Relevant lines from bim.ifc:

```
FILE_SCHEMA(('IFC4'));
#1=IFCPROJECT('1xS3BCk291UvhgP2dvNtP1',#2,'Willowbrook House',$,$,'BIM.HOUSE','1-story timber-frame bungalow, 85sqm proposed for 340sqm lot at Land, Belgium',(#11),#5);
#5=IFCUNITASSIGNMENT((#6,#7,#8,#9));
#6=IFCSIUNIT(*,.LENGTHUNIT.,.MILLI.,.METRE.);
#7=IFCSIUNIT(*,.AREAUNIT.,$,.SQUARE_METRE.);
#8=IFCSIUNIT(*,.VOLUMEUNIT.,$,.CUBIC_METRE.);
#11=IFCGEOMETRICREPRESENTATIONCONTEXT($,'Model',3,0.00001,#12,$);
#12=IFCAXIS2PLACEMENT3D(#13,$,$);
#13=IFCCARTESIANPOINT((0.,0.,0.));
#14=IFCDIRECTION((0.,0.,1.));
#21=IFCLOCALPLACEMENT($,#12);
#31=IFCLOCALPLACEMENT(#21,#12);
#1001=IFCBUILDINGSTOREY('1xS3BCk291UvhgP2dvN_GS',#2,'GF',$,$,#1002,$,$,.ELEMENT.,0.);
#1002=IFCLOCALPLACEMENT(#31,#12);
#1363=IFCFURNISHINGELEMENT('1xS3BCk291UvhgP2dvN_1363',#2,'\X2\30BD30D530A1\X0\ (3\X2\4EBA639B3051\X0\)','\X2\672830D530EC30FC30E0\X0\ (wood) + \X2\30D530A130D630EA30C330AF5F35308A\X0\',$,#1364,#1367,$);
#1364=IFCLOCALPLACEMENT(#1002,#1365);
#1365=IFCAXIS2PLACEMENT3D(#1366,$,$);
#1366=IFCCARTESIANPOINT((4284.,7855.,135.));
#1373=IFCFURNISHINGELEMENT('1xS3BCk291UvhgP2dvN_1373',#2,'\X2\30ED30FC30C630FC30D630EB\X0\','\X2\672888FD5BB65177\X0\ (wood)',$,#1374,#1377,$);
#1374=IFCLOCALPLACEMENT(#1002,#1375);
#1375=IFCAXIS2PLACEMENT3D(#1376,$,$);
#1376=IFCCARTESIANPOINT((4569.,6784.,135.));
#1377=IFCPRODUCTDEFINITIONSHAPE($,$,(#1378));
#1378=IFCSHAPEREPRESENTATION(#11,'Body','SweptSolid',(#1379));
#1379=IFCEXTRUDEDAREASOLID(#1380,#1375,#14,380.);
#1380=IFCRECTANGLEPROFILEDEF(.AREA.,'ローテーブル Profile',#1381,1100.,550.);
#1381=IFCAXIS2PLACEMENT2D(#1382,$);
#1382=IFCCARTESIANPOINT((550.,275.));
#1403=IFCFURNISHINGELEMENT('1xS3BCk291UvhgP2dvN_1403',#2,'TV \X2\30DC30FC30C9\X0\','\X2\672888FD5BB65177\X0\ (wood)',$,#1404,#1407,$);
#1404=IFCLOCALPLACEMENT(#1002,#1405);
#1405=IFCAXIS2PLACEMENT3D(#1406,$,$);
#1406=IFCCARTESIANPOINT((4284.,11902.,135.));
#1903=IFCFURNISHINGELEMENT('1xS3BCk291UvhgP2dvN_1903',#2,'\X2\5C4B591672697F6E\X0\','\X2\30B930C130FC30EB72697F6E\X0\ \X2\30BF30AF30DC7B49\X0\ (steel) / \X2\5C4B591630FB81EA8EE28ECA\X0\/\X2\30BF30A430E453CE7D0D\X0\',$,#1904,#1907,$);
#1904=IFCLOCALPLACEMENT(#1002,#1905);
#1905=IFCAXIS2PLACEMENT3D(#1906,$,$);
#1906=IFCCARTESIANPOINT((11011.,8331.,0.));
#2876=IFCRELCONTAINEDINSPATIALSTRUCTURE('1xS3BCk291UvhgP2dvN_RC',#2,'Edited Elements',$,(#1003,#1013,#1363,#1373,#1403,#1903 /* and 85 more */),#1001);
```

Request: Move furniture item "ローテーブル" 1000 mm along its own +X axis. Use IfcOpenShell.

```python
import ifcopenshell
import ifcopenshell.api.geometry
import ifcopenshell.util.placement
import ifcopenshell.util.unit

model = ifcopenshell.open("bim.ifc")
unit_scale = ifcopenshell.util.unit.calculate_unit_scale(model)

item = model.by_id(1373)
matrix = ifcopenshell.util.placement.get_local_placement(item.ObjectPlacement)
matrix[:3, 3] += matrix[:3, 0] * 1 / unit_scale
ifcopenshell.api.geometry.edit_object_placement(model, product=item, matrix=matrix, is_si=False)

print(ifcopenshell.util.placement.get_local_placement(item.ObjectPlacement).round(3) + 0.0)

model.write("bim-out.ifc")
```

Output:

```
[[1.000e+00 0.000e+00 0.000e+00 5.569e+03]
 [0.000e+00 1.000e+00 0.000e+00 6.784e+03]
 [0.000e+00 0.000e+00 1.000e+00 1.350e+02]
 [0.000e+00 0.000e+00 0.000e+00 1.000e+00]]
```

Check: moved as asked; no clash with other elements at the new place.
